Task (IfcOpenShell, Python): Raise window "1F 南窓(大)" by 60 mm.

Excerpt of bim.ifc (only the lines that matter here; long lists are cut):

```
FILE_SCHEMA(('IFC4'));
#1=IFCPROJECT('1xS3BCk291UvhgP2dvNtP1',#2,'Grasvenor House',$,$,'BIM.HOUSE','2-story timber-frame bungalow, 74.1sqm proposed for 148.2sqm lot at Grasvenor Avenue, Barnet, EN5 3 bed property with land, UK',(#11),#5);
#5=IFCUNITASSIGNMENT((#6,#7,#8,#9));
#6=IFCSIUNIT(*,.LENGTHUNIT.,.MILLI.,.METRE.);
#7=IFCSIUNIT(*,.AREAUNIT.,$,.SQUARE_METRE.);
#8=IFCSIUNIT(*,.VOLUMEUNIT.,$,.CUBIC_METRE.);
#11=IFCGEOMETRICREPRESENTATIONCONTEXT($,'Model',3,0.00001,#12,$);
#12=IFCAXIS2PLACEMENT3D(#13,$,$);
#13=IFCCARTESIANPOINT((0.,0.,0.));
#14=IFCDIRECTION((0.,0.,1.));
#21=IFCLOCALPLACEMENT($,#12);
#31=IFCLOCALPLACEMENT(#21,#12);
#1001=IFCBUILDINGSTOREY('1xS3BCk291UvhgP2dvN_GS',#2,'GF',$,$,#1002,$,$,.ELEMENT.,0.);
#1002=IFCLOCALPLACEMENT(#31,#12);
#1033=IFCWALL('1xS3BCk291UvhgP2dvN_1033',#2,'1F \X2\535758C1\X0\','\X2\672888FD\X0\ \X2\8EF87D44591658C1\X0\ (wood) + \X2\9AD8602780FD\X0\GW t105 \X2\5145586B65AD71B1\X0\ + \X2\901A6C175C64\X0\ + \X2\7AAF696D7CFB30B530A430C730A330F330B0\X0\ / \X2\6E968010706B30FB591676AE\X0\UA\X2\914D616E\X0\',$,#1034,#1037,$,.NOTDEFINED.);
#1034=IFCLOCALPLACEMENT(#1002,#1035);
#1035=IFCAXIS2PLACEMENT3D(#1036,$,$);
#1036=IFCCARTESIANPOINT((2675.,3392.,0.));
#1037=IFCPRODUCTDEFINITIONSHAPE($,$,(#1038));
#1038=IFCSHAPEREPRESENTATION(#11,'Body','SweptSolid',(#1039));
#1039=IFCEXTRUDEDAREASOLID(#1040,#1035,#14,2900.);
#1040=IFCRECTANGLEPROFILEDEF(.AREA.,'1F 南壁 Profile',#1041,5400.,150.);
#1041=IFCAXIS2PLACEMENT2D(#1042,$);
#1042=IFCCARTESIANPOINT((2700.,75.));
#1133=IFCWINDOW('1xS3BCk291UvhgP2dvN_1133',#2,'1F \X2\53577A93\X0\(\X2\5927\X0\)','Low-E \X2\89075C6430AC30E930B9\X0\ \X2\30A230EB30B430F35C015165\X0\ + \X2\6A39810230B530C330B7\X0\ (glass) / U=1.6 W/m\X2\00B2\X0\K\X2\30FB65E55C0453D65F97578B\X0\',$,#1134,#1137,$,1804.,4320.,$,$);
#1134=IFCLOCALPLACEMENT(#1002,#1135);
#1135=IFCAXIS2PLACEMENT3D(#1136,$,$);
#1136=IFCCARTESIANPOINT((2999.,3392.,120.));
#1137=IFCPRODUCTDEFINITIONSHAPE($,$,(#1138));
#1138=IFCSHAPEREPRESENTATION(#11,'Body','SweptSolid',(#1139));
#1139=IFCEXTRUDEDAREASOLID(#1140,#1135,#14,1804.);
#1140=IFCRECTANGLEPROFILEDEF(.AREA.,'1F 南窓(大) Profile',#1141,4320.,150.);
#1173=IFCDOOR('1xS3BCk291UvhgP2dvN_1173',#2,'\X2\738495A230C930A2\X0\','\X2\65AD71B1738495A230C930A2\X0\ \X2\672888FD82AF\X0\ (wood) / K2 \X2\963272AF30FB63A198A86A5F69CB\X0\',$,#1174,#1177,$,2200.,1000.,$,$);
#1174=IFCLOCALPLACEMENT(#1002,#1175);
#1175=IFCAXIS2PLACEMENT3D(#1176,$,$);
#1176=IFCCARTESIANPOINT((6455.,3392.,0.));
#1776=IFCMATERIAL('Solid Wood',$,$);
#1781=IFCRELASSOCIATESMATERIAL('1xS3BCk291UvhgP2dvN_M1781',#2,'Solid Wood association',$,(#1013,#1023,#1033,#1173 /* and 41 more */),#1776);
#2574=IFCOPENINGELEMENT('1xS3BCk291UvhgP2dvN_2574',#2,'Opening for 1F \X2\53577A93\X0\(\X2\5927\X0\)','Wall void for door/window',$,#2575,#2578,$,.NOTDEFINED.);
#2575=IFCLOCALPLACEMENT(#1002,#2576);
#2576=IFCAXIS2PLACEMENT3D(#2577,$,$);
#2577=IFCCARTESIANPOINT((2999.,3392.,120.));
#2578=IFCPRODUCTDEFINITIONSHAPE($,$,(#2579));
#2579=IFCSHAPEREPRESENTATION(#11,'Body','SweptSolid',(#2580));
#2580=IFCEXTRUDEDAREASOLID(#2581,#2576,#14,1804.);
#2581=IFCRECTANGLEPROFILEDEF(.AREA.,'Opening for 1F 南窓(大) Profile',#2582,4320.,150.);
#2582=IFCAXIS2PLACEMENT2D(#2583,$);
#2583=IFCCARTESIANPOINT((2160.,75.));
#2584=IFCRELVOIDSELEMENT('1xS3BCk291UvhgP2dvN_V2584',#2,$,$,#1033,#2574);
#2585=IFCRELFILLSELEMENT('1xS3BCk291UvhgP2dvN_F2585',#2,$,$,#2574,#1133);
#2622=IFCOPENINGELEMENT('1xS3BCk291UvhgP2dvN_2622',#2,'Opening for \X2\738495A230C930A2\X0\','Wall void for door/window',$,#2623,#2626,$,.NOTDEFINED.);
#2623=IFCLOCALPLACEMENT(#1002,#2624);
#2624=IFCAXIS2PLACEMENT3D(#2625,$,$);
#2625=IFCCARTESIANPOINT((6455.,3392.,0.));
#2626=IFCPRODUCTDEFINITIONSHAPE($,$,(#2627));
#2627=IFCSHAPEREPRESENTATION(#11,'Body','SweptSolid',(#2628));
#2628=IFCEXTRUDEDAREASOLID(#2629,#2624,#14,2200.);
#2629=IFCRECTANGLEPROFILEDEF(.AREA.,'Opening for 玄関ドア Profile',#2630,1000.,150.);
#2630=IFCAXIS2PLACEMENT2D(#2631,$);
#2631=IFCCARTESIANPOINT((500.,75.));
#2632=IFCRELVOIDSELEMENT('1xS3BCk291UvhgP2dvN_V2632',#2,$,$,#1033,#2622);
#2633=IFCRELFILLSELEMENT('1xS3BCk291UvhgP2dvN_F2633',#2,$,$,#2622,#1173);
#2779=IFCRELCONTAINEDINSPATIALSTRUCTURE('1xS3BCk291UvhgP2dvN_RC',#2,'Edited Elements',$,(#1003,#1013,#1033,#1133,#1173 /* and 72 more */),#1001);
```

```python
import numpy as np
import ifcopenshell
import ifcopenshell.api.geometry
import ifcopenshell.util.placement
import ifcopenshell.util.unit

model = ifcopenshell.open("bim.ifc")
unit_scale = ifcopenshell.util.unit.calculate_unit_scale(model)

window = model.by_id(1133)
opening = window.FillsVoids[0].RelatingOpeningElement
dz = 0.06 / unit_scale

shift = np.array([0.0, 0.0, dz])
# The window is not placed relative to its opening, so move both.
for product in (opening, window):
    matrix = ifcopenshell.util.placement.get_local_placement(product.ObjectPlacement)
    matrix[:3, 3] += shift
    ifcopenshell.api.geometry.edit_object_placement(model, product=product, matrix=matrix, is_si=False)

print(f"moved by {dz * unit_scale:+.3f} m")

model.write("bim_edited.ifc")
```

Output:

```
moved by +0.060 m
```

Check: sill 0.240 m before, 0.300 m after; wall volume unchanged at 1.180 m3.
